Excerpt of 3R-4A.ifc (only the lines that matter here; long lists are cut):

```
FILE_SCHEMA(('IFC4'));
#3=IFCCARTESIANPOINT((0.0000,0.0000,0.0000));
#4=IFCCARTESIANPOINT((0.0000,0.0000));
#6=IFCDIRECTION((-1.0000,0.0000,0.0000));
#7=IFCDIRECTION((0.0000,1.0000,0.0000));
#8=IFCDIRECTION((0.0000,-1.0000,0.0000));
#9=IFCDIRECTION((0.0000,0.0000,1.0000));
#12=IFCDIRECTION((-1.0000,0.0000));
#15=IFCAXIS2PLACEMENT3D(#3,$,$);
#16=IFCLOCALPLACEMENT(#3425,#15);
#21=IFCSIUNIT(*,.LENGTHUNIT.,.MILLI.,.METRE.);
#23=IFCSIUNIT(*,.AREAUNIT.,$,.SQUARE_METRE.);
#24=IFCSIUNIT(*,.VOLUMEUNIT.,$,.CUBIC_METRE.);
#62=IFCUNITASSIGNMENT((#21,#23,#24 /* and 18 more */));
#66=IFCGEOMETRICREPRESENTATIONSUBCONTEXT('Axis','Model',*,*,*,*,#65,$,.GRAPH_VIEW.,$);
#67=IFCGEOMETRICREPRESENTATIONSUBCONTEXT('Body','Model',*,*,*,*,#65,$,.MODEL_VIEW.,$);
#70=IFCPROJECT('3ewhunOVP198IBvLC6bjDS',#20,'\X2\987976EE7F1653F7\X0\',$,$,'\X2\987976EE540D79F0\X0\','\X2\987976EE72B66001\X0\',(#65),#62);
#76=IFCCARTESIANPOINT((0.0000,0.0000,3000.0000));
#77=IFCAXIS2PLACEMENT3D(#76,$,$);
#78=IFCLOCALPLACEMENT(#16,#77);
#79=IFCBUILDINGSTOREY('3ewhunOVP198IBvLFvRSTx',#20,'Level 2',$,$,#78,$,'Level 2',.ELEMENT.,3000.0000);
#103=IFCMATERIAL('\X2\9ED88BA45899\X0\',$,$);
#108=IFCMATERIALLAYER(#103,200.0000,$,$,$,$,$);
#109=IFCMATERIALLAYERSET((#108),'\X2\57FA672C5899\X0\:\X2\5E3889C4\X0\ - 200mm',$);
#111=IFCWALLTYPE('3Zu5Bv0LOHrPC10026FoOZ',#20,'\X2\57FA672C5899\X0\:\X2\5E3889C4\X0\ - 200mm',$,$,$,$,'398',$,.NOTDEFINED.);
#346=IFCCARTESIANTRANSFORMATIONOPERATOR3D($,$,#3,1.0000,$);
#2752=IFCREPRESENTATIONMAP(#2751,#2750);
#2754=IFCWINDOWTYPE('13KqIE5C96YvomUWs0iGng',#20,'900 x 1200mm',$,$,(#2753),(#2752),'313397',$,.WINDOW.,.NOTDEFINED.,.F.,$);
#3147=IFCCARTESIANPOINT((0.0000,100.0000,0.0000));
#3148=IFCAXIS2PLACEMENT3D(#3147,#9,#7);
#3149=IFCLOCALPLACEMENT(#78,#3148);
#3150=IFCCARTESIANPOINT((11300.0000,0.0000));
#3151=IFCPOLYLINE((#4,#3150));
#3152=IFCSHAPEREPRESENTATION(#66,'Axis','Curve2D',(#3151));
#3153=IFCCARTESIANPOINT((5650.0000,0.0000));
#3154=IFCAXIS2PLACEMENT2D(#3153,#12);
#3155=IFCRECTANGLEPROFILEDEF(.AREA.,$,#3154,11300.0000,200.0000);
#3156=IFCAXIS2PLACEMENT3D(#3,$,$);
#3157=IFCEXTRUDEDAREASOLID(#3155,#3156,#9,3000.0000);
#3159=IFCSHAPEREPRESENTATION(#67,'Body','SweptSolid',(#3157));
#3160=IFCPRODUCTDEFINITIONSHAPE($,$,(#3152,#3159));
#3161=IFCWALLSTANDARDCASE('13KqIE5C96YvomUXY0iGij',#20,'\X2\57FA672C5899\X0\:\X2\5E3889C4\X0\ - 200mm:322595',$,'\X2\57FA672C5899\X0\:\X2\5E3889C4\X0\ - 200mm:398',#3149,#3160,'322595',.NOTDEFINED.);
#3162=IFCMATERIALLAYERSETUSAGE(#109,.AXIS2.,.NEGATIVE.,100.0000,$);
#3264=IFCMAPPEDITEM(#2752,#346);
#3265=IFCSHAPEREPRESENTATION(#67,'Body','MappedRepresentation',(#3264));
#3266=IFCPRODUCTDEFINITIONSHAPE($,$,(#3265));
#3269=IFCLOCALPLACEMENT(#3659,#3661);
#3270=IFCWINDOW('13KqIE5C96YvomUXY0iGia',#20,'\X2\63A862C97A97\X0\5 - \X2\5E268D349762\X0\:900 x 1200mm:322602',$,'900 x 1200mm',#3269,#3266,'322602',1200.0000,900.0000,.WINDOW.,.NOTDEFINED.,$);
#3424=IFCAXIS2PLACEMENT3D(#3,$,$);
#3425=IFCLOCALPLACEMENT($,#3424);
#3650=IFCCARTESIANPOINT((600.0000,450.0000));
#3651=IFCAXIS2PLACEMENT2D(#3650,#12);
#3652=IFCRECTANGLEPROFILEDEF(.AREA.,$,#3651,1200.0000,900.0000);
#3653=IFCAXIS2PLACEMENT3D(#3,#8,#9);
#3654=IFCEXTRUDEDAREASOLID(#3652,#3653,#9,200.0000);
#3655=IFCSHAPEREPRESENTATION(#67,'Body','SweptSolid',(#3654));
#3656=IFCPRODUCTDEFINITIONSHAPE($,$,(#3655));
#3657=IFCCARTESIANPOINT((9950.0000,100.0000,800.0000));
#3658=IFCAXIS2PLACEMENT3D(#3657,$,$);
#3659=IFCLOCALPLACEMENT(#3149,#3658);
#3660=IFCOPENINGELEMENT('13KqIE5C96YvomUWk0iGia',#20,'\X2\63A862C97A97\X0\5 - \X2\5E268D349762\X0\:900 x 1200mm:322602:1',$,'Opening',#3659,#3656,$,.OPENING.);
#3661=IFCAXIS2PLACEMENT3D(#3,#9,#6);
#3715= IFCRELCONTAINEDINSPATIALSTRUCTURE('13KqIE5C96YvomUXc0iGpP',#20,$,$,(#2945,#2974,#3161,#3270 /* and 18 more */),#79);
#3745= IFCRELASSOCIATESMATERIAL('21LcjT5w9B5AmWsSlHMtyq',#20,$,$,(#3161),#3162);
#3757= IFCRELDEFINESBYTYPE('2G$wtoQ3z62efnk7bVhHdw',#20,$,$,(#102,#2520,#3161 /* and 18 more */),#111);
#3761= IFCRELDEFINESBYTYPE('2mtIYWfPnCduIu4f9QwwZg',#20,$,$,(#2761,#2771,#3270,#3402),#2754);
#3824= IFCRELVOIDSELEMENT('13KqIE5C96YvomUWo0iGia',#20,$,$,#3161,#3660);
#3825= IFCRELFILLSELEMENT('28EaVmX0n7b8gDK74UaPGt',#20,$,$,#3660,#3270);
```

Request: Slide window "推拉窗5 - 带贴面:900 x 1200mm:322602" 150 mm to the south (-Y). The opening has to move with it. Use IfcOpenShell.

```python
import ifcopenshell
import ifcopenshell.api.geometry
import ifcopenshell.util.placement

model = ifcopenshell.open("3R-4A.ifc")

window = model.by_id(3270)
opening = window.FillsVoids[0].RelatingOpeningElement
wall = opening.VoidsElements[0].RelatingBuildingElement

wall_matrix = ifcopenshell.util.placement.get_local_placement(wall.ObjectPlacement)
shift = wall_matrix[:3, 0] * -150.0
before = ifcopenshell.util.placement.get_local_placement(window.ObjectPlacement)[:3, 3].copy()

# The window is placed relative to its opening, so it follows when the opening moves.
matrix = ifcopenshell.util.placement.get_local_placement(opening.ObjectPlacement)
matrix[:3, 3] += shift
ifcopenshell.api.geometry.edit_object_placement(
    model, product=opening, matrix=matrix, is_si=False, should_transform_children=True
)

after = ifcopenshell.util.placement.get_local_placement(window.ObjectPlacement)[:3, 3]
print("window moved by", (after - before).round(3) + 0.0)

model.write("3R-4A_edited.ifc")
```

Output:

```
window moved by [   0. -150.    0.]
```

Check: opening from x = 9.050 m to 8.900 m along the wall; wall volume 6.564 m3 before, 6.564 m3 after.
